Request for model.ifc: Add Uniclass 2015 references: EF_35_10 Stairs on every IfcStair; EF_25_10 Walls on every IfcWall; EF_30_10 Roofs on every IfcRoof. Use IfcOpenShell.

First a look at what the model holds.

```python
import ifcopenshell

model = ifcopenshell.open("model.ifc")
print(model.schema)
print("classifications:", [c.Name for c in model.by_type("IfcClassification")])
for ifc_class in ("IfcDoor", "IfcRoof", "IfcStair", "IfcWall", "IfcWindow"):
    print(ifc_class, len(model.by_type(ifc_class)))
```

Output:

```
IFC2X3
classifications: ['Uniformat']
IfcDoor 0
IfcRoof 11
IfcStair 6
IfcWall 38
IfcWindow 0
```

```python
import ifcopenshell
import ifcopenshell.api.classification

model = ifcopenshell.open("model.ifc")

# IFC2X3 requires Source and Edition and has no link from the project to the system.
system = model.create_entity("IfcClassification", Source="NBS", Edition="2015", Name="Uniclass 2015")

codes = {
    "IfcStair": ("EF_35_10", "Stairs"),
    "IfcWall": ("EF_25_10", "Walls"),
    "IfcRoof": ("EF_30_10", "Roofs"),
}
for ifc_class, (code, name) in codes.items():
    products = model.by_type(ifc_class)
    ifcopenshell.api.classification.add_reference(
        model, products=products, classification=system, identification=code, name=name
    )
    print(code, len(products))

model.write("model_v2.ifc")
```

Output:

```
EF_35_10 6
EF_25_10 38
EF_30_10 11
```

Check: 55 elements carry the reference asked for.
